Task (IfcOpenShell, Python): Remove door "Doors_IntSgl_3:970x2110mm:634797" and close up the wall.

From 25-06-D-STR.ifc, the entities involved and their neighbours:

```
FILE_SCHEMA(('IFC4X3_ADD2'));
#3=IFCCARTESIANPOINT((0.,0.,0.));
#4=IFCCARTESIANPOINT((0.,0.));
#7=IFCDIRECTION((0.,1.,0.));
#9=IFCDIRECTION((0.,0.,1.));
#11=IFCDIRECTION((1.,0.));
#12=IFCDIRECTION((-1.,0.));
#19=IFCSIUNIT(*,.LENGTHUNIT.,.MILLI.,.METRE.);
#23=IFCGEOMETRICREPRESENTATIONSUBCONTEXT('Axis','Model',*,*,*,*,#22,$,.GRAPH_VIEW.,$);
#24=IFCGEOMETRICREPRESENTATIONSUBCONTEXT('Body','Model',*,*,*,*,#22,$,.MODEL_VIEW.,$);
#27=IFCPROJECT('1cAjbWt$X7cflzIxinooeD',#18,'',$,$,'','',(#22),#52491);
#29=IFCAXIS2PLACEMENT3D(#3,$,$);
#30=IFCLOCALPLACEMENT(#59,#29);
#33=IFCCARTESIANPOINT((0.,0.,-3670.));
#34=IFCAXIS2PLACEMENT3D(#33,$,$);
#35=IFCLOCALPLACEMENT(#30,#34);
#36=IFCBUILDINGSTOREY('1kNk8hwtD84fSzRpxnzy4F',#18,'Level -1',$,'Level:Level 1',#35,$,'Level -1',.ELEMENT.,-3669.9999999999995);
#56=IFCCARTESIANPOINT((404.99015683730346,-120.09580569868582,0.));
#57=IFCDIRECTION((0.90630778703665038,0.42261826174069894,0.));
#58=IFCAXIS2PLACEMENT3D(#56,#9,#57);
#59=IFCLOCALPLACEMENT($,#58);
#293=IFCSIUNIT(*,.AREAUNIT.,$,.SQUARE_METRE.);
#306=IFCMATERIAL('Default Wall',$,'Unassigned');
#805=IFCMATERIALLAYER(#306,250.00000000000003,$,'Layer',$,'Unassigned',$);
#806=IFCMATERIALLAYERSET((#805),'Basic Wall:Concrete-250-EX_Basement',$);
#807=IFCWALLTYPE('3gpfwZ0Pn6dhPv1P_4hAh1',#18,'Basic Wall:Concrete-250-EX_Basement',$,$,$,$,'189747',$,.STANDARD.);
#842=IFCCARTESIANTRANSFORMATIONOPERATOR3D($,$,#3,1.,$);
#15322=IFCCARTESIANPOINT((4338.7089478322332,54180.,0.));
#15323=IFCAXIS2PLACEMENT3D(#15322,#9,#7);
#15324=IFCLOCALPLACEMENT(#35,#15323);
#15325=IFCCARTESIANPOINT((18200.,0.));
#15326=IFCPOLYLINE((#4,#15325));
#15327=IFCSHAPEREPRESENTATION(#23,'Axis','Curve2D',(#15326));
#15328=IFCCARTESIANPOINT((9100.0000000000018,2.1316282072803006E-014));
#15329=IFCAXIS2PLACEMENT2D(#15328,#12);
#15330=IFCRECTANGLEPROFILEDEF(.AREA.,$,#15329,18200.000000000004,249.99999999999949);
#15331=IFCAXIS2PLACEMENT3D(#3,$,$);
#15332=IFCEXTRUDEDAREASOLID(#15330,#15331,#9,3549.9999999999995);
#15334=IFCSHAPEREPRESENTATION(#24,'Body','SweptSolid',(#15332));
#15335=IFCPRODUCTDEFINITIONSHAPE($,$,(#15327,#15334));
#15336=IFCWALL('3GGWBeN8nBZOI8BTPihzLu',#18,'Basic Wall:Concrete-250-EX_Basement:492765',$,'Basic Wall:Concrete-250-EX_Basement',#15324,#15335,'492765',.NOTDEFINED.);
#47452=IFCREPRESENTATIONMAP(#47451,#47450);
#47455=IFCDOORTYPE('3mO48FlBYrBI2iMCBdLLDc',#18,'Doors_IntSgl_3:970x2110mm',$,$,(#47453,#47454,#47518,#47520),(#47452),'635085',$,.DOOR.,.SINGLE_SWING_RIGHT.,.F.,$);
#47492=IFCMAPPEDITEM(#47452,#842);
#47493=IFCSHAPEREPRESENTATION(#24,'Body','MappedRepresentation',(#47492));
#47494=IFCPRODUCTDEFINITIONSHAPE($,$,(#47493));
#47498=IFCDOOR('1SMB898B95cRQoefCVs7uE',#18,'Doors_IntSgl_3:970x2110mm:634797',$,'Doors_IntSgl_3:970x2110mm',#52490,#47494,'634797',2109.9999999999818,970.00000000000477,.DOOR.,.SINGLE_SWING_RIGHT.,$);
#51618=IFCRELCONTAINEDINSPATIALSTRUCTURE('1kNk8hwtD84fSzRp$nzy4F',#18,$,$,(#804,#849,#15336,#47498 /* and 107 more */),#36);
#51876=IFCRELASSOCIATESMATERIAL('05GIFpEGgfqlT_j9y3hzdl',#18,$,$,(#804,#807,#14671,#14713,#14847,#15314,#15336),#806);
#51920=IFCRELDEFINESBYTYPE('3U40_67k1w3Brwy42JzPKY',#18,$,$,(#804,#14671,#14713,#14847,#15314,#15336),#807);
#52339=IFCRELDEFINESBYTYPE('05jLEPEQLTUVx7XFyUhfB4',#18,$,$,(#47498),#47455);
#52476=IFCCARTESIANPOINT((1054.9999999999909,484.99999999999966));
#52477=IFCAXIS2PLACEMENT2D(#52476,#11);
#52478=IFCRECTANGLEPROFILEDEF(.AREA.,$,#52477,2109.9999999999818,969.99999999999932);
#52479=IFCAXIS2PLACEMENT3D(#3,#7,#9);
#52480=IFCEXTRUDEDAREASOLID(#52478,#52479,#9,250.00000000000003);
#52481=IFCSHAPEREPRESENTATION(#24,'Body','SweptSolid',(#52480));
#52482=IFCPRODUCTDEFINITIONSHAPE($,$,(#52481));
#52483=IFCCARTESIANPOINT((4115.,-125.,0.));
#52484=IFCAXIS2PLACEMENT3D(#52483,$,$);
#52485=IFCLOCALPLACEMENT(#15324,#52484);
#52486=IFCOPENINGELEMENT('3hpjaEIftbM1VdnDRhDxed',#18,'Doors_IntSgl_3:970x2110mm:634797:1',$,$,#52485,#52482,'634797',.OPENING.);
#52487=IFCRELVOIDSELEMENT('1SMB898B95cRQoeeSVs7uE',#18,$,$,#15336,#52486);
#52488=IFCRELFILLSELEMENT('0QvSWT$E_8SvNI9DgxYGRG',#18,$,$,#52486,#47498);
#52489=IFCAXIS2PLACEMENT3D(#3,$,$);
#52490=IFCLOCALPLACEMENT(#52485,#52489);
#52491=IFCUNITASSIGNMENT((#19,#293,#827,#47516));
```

```python
import ifcopenshell
import ifcopenshell.api.feature
import ifcopenshell.api.root
import ifcopenshell.geom
import ifcopenshell.util.shape

model = ifcopenshell.open("25-06-D-STR.ifc")
settings = ifcopenshell.geom.settings()


def volume(element):
    """Net volume in cubic metres, openings subtracted."""
    shape = ifcopenshell.geom.create_shape(settings, element)
    return ifcopenshell.util.shape.get_volume(shape.geometry)


door = model.by_guid("1SMB898B95cRQoefCVs7uE")
opening = door.FillsVoids[0].RelatingOpeningElement
wall = opening.VoidsElements[0].RelatingBuildingElement
before = volume(wall)

ifcopenshell.api.root.remove_product(model, product=door)
ifcopenshell.api.feature.remove_feature(model, feature=opening)

after = volume(wall)

print(f"wall volume {before:.3f} -> {after:.3f} m3")

model.write("25-06-D-STR_edited.ifc")
```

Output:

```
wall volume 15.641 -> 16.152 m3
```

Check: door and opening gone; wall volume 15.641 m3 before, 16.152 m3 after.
